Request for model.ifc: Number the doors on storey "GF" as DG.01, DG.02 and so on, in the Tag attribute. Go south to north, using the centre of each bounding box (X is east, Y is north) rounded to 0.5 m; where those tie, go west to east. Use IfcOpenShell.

First a look at what the model holds.

```python
import ifcopenshell
import ifcopenshell.util.element
import ifcopenshell.util.placement

model = ifcopenshell.open("model.ifc")
print(model.schema)
storey = next(s for s in model.by_type("IfcBuildingStorey") if s.Name == "GF")
doors = [e for e in ifcopenshell.util.element.get_decomposition(storey) if e.is_a("IfcDoor")]
for e in sorted(doors, key=lambda e: e.id()):
    origin = ifcopenshell.util.placement.get_local_placement(e.ObjectPlacement)[:3, 3]
    print(e.id(), e.Tag, e.Name, origin.round(2) + 0.0, sep=" | ")
```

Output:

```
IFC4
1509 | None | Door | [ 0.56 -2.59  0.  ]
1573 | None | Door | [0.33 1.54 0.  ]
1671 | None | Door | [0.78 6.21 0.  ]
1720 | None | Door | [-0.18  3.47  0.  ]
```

```python
import ifcopenshell
import ifcopenshell.geom
import ifcopenshell.util.element
import ifcopenshell.util.shape

model = ifcopenshell.open("model.ifc")
settings = ifcopenshell.geom.settings()
settings.set("use-world-coords", True)


def centre(element):
    shape = ifcopenshell.geom.create_shape(settings, element)
    return ifcopenshell.util.shape.get_bbox_centroid(shape.geometry)


storey = next(s for s in model.by_type("IfcBuildingStorey") if s.Name == "GF")
doors = [e for e in ifcopenshell.util.element.get_decomposition(storey) if e.is_a("IfcDoor")]

# Insertion points can sit at a corner or the storey origin, so sort by the geometry (in metres).
centres = {e: centre(e) for e in doors}
doors.sort(key=lambda e: (round(centres[e][1] / 0.5), centres[e][0]))

for i, e in enumerate(doors, start=1):
    number = f"DG.{i:02d}"
    e.Tag = number
    print(e.id(), number)

model.write("model_v2.ifc")
```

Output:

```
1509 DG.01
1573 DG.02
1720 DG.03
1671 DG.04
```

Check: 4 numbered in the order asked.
